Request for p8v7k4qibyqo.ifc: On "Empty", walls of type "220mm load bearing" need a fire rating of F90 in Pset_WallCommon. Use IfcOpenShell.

First a look at what the model holds.

```python
import ifcopenshell
import ifcopenshell.util.element

model = ifcopenshell.open("p8v7k4qibyqo.ifc")
print(model.schema)
storey = next(s for s in model.by_type("IfcBuildingStorey") if s.Name == "Empty")
walls = [e for e in ifcopenshell.util.element.get_decomposition(storey) if e.is_a("IfcWall")]
seen = {}
for e in walls:
    element_type = ifcopenshell.util.element.get_type(e)
    key = (element_type.Name if element_type != e and element_type else None, ifcopenshell.util.element.get_pset(e, "Pset_WallCommon", "FireRating"))
    seen[key] = seen.get(key, 0) + 1
for (name, value), count in sorted(seen.items(), key=str):
    print(count, "x", name, "|", value)
```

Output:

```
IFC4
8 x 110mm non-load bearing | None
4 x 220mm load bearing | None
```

```python
import ifcopenshell
import ifcopenshell.api.pset
import ifcopenshell.util.element

model = ifcopenshell.open("p8v7k4qibyqo.ifc")

storey = next(s for s in model.by_type("IfcBuildingStorey") if s.Name == "Empty")
walls = [e for e in ifcopenshell.util.element.get_decomposition(storey) if e.is_a("IfcWall")]

count = 0
for e in walls:
    element_type = ifcopenshell.util.element.get_type(e)
    if element_type in (None, e) or element_type.Name != "220mm load bearing":
        continue
    # add_pset returns the element's existing set when there is one.
    pset = ifcopenshell.api.pset.add_pset(model, product=e, name="Pset_WallCommon")
    ifcopenshell.api.pset.edit_pset(model, pset=pset, properties={"FireRating": "F90"})
    count += 1

print(count, "walls updated")

model.write("p8v7k4qibyqo_updated.ifc")
```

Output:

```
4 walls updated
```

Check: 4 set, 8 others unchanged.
